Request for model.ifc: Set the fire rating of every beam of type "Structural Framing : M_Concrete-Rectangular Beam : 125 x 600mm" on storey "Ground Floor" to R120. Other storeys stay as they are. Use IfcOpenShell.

First a look at what the model holds.

```python
import ifcopenshell
import ifcopenshell.util.element

model = ifcopenshell.open("model.ifc")
print(model.schema)
storey = next(s for s in model.by_type("IfcBuildingStorey") if s.Name == "Ground Floor")
beams = [e for e in ifcopenshell.util.element.get_decomposition(storey) if e.is_a("IfcBeam")]
seen = {}
for e in beams:
    element_type = ifcopenshell.util.element.get_type(e)
    key = (element_type.Name if element_type != e and element_type else None, ifcopenshell.util.element.get_pset(e, "Pset_BeamCommon", "FireRating"))
    seen[key] = seen.get(key, 0) + 1
for (name, value), count in sorted(seen.items(), key=str):
    print(count, "x", name, "|", value)
```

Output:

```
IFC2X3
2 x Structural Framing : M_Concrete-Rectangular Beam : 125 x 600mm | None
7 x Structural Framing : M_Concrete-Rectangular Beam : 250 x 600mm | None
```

```python
import ifcopenshell
import ifcopenshell.api.pset
import ifcopenshell.util.element

model = ifcopenshell.open("model.ifc")

storey = next(s for s in model.by_type("IfcBuildingStorey") if s.Name == "Ground Floor")
beams = [e for e in ifcopenshell.util.element.get_decomposition(storey) if e.is_a("IfcBeam")]

count = 0
for e in beams:
    element_type = ifcopenshell.util.element.get_type(e)
    if element_type in (None, e) or element_type.Name != "Structural Framing : M_Concrete-Rectangular Beam : 125 x 600mm":
        continue
    # add_pset returns the element's existing set when there is one.
    pset = ifcopenshell.api.pset.add_pset(model, product=e, name="Pset_BeamCommon")
    ifcopenshell.api.pset.edit_pset(model, pset=pset, properties={"FireRating": "R120"})
    count += 1

print(count, "beams updated")

model.write("model-out.ifc")
```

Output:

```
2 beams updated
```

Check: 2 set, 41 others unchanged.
